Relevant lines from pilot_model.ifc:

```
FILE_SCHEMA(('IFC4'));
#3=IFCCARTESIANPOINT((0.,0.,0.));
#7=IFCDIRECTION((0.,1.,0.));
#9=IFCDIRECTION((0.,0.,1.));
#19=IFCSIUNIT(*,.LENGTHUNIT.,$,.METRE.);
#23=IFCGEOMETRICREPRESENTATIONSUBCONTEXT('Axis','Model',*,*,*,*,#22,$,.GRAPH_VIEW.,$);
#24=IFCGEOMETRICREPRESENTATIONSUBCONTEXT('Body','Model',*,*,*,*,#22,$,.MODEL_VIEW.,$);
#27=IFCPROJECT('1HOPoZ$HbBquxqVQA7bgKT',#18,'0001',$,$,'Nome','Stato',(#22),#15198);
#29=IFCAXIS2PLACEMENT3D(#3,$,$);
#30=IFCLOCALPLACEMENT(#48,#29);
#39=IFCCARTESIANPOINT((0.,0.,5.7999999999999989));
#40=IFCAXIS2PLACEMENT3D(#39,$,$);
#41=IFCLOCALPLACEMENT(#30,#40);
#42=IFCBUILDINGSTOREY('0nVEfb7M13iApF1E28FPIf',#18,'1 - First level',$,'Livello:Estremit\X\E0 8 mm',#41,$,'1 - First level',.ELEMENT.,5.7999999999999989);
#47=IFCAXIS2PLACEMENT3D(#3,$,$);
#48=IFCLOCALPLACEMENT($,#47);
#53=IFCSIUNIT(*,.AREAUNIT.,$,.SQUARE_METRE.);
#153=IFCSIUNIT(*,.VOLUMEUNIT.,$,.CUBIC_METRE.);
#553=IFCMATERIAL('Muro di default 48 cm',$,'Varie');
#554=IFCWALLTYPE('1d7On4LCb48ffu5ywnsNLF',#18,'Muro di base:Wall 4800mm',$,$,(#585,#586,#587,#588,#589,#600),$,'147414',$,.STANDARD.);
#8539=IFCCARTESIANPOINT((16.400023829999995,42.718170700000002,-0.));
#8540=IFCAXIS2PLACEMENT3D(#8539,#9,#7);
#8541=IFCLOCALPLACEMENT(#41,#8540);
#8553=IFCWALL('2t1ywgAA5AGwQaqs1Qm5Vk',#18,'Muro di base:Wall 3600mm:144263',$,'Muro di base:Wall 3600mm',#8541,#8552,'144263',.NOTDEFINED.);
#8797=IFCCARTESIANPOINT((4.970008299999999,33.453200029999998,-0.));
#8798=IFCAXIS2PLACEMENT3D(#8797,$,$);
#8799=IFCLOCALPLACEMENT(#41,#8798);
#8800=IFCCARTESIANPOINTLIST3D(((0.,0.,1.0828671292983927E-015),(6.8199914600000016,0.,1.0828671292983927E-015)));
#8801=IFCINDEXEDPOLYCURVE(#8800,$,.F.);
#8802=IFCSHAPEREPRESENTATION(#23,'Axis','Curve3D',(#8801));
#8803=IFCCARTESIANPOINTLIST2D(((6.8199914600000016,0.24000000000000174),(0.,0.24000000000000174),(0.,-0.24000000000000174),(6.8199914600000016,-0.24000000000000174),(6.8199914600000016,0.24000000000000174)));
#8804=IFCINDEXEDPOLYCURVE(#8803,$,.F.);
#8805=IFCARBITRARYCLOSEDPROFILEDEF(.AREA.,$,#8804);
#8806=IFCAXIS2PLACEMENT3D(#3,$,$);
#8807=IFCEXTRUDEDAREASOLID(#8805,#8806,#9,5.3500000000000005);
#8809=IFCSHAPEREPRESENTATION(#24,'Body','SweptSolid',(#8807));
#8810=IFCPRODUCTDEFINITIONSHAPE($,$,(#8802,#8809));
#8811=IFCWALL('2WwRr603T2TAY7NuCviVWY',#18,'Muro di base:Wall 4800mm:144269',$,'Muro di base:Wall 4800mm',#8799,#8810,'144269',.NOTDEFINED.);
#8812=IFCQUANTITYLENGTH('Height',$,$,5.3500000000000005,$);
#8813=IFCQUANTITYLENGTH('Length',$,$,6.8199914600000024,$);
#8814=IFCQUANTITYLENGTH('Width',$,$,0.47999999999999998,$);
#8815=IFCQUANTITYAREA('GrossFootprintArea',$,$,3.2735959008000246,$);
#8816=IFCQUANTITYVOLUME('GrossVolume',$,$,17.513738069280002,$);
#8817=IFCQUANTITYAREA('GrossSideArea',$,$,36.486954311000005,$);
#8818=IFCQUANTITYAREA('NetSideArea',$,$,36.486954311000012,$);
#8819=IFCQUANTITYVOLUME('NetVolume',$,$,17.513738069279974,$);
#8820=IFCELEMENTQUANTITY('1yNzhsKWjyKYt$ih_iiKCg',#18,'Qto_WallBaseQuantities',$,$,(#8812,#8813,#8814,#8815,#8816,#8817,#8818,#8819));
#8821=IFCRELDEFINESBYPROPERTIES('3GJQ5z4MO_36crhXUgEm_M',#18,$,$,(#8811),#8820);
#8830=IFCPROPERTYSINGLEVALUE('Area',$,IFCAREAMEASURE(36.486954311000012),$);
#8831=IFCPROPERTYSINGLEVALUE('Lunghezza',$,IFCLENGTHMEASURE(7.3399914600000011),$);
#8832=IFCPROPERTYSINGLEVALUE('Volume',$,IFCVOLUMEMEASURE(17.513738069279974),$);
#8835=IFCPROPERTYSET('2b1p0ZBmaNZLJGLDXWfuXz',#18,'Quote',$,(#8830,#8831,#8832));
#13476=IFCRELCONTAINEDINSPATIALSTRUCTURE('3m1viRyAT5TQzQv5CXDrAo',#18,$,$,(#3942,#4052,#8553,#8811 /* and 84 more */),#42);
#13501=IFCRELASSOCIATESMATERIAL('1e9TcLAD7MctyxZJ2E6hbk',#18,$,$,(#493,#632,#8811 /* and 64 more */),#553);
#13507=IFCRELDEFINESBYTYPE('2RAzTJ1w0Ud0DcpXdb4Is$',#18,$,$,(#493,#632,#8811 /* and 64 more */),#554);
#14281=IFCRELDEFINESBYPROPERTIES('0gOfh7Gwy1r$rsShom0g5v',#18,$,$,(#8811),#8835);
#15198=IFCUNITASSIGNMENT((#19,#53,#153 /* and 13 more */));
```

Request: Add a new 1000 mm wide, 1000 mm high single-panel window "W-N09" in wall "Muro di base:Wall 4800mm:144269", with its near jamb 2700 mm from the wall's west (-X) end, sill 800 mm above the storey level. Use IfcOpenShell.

```python
import numpy as np
import ifcopenshell
import ifcopenshell.api.feature
import ifcopenshell.api.geometry
import ifcopenshell.api.pset
import ifcopenshell.api.root
import ifcopenshell.api.spatial
import ifcopenshell.geom
import ifcopenshell.util.element
import ifcopenshell.util.placement
import ifcopenshell.util.representation
import ifcopenshell.util.shape
import ifcopenshell.util.unit

model = ifcopenshell.open("pilot_model.ifc")
unit_scale = ifcopenshell.util.unit.calculate_unit_scale(model)
area_scale = ifcopenshell.util.unit.calculate_unit_scale(model, "AREAUNIT")
volume_scale = ifcopenshell.util.unit.calculate_unit_scale(model, "VOLUMEUNIT")
settings = ifcopenshell.geom.settings()


def volume(element):
    """Net volume in cubic metres, openings subtracted."""
    shape = ifcopenshell.geom.create_shape(settings, element)
    return ifcopenshell.util.shape.get_volume(shape.geometry)


wall = model.by_guid("2WwRr603T2TAY7NuCviVWY")
storey = ifcopenshell.util.element.get_container(wall, ifc_class="IfcBuildingStorey")
context = ifcopenshell.util.representation.get_context(model, "Model", "Body", "MODEL_VIEW")
before = volume(wall)

width, height, from_end, sill = 1, 1, 2.7, 0.8  # metres

# The wall runs along its own X axis, and the end named is its -X end.
wall_shape = ifcopenshell.geom.create_shape(settings, wall)
x, y, z = ifcopenshell.util.shape.get_vertices(wall_shape.geometry).T
start = x.min() + from_end
face, thickness = float(y.min()), float(y.max() - y.min())
wall_matrix = ifcopenshell.util.placement.get_local_placement(wall.ObjectPlacement)
level = ifcopenshell.util.placement.get_local_placement(storey.ObjectPlacement)[2, 3]


def in_wall(x, y):
    """Placement at x, y metres in the wall's axes, at sill height."""
    matrix = wall_matrix.copy()
    matrix[:, 3] = wall_matrix @ np.array([x / unit_scale, y / unit_scale, 0.0, 1.0])
    matrix[2, 3] = level + sill / unit_scale
    return matrix


# Opening: a box that overshoots both wall faces by 50 mm.
opening = ifcopenshell.api.root.create_entity(model, ifc_class="IfcOpeningElement", predefined_type="OPENING")
box = ifcopenshell.api.geometry.add_wall_representation(
    model, context=context, length=width, height=height, thickness=thickness + 0.1
)
ifcopenshell.api.geometry.assign_representation(model, product=opening, representation=box)
ifcopenshell.api.geometry.edit_object_placement(model, product=opening, matrix=in_wall(start, face - 0.05), is_si=False)
ifcopenshell.api.feature.add_feature(model, feature=opening, element=wall)

window = ifcopenshell.api.root.create_entity(model, ifc_class="IfcWindow", name="W-N09", predefined_type="WINDOW")
window.OverallWidth, window.OverallHeight = width / unit_scale, height / unit_scale
window.PartitioningType = "SINGLE_PANEL"
body = ifcopenshell.api.geometry.add_window_representation(
    model,
    context=context,
    overall_width=window.OverallWidth,
    overall_height=window.OverallHeight,
    partition_type="SINGLE_PANEL",
)
ifcopenshell.api.geometry.assign_representation(model, product=window, representation=body)
ifcopenshell.api.spatial.assign_container(model, products=[window], relating_structure=storey)
ifcopenshell.api.feature.add_filling(model, opening=opening, element=window)

# Centre the window in the wall's thickness.
ifcopenshell.api.geometry.edit_object_placement(model, product=window, matrix=in_wall(start, face), is_si=False)
window_shape = ifcopenshell.geom.create_shape(settings, window)
depth = ifcopenshell.util.shape.get_vertices(window_shape.geometry)[:, 1]
offset = face + thickness / 2 - (depth.min() + depth.max()) / 2
ifcopenshell.api.geometry.edit_object_placement(model, product=window, matrix=in_wall(start, offset), is_si=False)

after = volume(wall)

# Update the wall's stored quantities.
qto = model.by_id(ifcopenshell.util.element.get_pset(wall, "Qto_WallBaseQuantities", should_inherit=False)["id"])
ifcopenshell.api.pset.edit_qto(model, qto=qto, properties={
    "NetSideArea": after / thickness / area_scale,
    "NetVolume": after / volume_scale,
})
pset = model.by_id(ifcopenshell.util.element.get_pset(wall, "Quote", should_inherit=False)["id"])
ifcopenshell.api.pset.edit_pset(model, pset=pset, properties={
    "Area": model.create_entity("IfcAreaMeasure", after / thickness / area_scale),
    "Volume": model.create_entity("IfcVolumeMeasure", after / volume_scale),
})

print(f"wall volume {before:.3f} -> {after:.3f} m3")

model.write("pilot_model_edited.ifc")
```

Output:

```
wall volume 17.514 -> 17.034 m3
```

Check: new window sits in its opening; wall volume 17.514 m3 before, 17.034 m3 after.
